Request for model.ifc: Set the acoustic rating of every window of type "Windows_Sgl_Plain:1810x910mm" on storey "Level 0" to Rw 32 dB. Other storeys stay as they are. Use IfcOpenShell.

First a look at what the model holds.

```python
import ifcopenshell
import ifcopenshell.util.element

model = ifcopenshell.open("model.ifc")
print(model.schema)
storey = next(s for s in model.by_type("IfcBuildingStorey") if s.Name == "Level 0")
windows = [e for e in ifcopenshell.util.element.get_decomposition(storey) if e.is_a("IfcWindow")]
seen = {}
for e in windows:
    element_type = ifcopenshell.util.element.get_type(e)
    key = (element_type.Name if element_type != e and element_type else None, ifcopenshell.util.element.get_pset(e, "Pset_WindowCommon", "AcousticRating"))
    seen[key] = seen.get(key, 0) + 1
for (name, value), count in sorted(seen.items(), key=str):
    print(count, "x", name, "|", value)
```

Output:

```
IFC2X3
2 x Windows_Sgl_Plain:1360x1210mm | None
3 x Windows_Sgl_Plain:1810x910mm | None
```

```python
import ifcopenshell
import ifcopenshell.api.pset
import ifcopenshell.util.element

model = ifcopenshell.open("model.ifc")

storey = next(s for s in model.by_type("IfcBuildingStorey") if s.Name == "Level 0")
windows = [e for e in ifcopenshell.util.element.get_decomposition(storey) if e.is_a("IfcWindow")]

count = 0
for e in windows:
    element_type = ifcopenshell.util.element.get_type(e)
    if element_type in (None, e) or element_type.Name != "Windows_Sgl_Plain:1810x910mm":
        continue
    # add_pset returns the element's existing set when there is one.
    pset = ifcopenshell.api.pset.add_pset(model, product=e, name="Pset_WindowCommon")
    ifcopenshell.api.pset.edit_pset(model, pset=pset, properties={"AcousticRating": "Rw 32 dB"})
    count += 1

print(count, "windows updated")

model.write("model_updated.ifc")
```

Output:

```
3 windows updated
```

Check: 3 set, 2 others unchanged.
